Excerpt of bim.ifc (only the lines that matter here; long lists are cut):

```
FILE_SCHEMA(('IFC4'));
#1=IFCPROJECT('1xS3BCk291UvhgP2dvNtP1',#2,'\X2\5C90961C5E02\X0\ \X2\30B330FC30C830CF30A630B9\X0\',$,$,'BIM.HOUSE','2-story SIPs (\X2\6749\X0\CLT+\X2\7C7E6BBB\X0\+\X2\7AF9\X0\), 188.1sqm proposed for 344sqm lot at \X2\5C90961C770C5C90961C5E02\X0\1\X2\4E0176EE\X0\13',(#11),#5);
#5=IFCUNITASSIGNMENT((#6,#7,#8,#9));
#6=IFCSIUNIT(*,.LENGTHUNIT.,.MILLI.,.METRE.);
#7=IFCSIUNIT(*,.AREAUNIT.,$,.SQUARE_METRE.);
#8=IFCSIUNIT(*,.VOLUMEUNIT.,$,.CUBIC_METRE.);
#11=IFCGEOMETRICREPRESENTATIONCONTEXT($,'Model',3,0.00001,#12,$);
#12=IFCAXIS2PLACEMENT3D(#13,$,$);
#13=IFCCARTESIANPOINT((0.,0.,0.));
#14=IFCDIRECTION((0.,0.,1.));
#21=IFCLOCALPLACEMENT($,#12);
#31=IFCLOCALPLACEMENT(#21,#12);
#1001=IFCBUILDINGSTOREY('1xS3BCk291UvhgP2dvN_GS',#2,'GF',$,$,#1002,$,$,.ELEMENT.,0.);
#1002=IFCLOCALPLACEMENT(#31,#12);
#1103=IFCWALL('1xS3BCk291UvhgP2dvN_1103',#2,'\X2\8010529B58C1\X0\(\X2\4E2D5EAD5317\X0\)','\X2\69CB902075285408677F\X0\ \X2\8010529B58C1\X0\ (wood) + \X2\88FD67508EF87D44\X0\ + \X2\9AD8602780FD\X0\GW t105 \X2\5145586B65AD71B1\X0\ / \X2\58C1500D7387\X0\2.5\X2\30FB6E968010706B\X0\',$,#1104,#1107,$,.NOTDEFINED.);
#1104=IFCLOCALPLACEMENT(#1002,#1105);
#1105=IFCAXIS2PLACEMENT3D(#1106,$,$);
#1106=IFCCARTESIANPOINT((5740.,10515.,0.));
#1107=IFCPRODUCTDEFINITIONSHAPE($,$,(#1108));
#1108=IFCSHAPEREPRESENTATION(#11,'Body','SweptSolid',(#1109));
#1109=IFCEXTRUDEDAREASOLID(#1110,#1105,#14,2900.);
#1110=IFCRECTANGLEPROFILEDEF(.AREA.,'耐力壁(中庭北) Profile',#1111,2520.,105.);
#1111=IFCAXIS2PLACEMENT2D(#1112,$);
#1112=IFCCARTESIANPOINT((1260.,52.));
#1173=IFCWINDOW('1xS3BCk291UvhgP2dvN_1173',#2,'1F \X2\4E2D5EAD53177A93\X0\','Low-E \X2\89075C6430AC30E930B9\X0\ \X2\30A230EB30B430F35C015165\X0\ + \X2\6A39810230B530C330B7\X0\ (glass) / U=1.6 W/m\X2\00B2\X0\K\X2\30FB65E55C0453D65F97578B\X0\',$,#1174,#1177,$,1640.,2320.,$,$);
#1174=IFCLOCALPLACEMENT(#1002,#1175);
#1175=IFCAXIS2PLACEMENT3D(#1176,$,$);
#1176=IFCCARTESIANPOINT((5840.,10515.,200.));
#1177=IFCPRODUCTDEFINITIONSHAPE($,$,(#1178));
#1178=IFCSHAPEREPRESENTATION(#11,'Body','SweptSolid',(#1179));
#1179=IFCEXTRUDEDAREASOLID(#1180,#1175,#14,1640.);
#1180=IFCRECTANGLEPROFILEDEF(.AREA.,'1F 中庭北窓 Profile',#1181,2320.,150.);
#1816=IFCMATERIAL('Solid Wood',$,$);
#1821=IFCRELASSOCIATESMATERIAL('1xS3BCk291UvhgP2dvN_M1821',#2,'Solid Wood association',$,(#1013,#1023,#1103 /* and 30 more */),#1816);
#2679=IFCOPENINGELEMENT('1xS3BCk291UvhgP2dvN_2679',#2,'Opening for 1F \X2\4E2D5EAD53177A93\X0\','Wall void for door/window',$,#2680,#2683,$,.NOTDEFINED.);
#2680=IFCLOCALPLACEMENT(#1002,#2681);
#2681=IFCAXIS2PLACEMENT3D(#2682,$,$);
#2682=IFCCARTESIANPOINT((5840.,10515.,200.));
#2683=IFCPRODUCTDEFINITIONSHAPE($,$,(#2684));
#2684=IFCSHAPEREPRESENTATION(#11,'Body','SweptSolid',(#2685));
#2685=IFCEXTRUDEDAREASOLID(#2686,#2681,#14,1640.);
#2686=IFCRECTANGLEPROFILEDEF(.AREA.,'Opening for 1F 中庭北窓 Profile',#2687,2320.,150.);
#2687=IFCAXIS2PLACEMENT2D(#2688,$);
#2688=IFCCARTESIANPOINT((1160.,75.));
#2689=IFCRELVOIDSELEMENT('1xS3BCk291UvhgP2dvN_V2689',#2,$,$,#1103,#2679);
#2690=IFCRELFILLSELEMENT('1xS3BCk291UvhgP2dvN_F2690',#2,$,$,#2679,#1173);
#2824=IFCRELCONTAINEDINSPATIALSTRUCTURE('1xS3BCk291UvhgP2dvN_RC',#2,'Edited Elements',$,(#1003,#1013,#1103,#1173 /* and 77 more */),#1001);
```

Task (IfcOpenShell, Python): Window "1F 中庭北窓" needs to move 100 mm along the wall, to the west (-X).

```python
import ifcopenshell
import ifcopenshell.api.geometry
import ifcopenshell.util.placement

model = ifcopenshell.open("bim.ifc")

window = model.by_guid("1xS3BCk291UvhgP2dvN_1173")
opening = window.FillsVoids[0].RelatingOpeningElement
wall = opening.VoidsElements[0].RelatingBuildingElement

wall_matrix = ifcopenshell.util.placement.get_local_placement(wall.ObjectPlacement)
shift = wall_matrix[:3, 0] * -100.0
before = ifcopenshell.util.placement.get_local_placement(window.ObjectPlacement)[:3, 3].copy()

# The window is not placed relative to its opening, so move both.
for product in (opening, window):
    matrix = ifcopenshell.util.placement.get_local_placement(product.ObjectPlacement)
    matrix[:3, 3] += shift
    ifcopenshell.api.geometry.edit_object_placement(model, product=product, matrix=matrix, is_si=False)

after = ifcopenshell.util.placement.get_local_placement(window.ObjectPlacement)[:3, 3]
print("window moved by", (after - before).round(3) + 0.0)

model.write("bim_updated.ifc")
```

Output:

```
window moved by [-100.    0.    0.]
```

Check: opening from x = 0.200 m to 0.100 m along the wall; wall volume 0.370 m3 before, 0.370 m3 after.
